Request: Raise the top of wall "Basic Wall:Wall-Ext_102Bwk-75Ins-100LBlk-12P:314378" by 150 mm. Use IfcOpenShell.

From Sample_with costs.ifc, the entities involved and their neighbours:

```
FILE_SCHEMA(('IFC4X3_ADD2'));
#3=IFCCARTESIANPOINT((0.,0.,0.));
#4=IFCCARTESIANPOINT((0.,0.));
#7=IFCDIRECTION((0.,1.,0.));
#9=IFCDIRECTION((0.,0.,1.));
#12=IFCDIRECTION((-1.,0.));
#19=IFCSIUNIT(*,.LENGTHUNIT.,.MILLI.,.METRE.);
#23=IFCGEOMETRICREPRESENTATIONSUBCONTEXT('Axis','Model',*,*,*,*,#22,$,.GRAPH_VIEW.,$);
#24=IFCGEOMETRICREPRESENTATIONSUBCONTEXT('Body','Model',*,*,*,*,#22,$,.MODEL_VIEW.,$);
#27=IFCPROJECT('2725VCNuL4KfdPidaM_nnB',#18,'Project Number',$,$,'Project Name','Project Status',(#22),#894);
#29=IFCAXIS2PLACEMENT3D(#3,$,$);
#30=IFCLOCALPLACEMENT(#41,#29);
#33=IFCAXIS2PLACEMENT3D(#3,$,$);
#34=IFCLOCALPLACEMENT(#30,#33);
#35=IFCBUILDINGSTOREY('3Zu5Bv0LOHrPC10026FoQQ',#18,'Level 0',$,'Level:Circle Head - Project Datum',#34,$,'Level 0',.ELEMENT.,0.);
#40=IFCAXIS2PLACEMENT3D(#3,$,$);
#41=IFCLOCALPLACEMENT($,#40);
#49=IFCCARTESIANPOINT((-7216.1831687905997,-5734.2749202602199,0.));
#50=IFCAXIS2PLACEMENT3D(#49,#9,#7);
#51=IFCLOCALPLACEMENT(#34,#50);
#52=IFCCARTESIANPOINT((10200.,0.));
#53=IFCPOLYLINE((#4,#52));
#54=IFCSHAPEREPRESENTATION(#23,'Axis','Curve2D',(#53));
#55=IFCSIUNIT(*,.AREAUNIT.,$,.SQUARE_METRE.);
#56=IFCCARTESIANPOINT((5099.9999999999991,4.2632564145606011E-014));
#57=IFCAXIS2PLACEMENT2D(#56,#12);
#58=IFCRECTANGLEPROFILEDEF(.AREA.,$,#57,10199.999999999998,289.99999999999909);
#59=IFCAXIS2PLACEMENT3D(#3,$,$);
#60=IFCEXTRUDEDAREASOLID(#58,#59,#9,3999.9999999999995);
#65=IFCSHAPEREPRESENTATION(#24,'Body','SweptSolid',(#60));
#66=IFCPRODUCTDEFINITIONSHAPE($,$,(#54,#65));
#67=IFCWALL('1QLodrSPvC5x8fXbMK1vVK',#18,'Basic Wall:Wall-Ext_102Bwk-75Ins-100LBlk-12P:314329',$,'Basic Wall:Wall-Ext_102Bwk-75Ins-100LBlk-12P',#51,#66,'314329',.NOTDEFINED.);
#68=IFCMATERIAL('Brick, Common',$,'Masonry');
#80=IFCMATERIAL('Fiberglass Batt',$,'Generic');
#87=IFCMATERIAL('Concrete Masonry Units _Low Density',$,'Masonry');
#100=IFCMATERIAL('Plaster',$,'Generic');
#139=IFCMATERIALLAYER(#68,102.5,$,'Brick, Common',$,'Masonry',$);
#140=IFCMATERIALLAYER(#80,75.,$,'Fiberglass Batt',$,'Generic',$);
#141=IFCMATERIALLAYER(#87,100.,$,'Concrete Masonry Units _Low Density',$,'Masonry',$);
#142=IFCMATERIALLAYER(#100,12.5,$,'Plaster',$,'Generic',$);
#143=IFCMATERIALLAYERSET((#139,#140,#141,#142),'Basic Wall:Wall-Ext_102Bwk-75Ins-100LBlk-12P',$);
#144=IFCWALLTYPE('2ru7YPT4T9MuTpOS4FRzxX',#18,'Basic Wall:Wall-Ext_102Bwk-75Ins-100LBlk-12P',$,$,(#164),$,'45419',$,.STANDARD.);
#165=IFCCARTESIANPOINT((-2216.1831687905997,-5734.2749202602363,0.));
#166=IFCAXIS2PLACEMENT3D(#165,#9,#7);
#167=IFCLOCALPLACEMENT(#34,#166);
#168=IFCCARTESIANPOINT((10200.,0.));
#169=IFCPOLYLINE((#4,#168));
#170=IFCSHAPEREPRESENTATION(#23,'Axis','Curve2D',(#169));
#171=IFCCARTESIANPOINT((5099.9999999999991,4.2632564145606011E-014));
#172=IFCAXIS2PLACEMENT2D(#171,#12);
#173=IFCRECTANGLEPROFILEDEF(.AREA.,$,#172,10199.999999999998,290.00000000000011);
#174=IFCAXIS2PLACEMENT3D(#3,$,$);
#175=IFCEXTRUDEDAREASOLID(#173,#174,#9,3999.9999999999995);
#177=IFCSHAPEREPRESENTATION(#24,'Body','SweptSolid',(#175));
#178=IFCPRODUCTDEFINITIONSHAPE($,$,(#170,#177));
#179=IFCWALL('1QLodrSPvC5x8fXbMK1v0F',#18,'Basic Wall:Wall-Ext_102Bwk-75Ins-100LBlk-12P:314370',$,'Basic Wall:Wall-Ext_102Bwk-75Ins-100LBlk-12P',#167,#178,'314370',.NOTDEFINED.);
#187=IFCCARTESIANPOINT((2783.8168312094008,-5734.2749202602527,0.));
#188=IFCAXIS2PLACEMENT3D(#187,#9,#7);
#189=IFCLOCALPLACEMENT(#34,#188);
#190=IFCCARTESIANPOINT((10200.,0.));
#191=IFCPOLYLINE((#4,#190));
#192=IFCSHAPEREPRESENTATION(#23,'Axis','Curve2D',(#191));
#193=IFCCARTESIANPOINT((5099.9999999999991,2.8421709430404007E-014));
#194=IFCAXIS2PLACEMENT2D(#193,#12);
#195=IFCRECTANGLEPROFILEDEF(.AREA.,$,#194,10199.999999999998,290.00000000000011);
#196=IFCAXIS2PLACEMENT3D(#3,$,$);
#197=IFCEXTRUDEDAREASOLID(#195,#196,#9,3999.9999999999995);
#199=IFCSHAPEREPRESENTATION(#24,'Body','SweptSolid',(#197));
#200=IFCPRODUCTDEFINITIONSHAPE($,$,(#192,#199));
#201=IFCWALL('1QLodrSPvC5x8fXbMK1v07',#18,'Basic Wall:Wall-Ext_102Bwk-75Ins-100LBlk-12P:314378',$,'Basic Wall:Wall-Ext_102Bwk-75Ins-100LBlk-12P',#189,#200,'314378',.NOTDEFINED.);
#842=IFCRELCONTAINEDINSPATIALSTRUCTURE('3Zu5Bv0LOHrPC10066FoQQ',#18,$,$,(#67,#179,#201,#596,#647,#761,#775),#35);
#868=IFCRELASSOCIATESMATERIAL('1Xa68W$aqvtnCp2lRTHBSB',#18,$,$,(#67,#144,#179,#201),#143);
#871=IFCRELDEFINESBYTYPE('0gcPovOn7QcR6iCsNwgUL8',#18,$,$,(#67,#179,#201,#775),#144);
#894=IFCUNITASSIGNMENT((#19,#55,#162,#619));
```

```python
import ifcopenshell
import ifcopenshell.geom
import ifcopenshell.util.representation
import ifcopenshell.util.shape

model = ifcopenshell.open("Sample_with costs.ifc")
settings = ifcopenshell.geom.settings()


def volume(element):
    """Net volume in cubic metres, openings subtracted."""
    shape = ifcopenshell.geom.create_shape(settings, element)
    return ifcopenshell.util.shape.get_volume(shape.geometry)


wall = model.by_guid("1QLodrSPvC5x8fXbMK1v07")
before = volume(wall)

body = ifcopenshell.util.representation.get_representation(wall, "Model", "Body")
solid = body.Items[0]
old_height = solid.Depth
solid.Depth += 150.0
after = volume(wall)

print(f"height {old_height:g} -> {solid.Depth:g}, volume {before:.3f} -> {after:.3f} m3")

model.write("Sample_with costs_edited.ifc")
```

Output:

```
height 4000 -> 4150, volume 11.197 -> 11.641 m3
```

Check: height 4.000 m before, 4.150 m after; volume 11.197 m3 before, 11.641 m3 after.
